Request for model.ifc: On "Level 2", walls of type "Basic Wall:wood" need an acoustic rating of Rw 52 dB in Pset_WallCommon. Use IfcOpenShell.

First a look at what the model holds.

```python
import ifcopenshell
import ifcopenshell.util.element

model = ifcopenshell.open("model.ifc")
print(model.schema)
storey = next(s for s in model.by_type("IfcBuildingStorey") if s.Name == "Level 2")
walls = [e for e in ifcopenshell.util.element.get_decomposition(storey) if e.is_a("IfcWall")]
seen = {}
for e in walls:
    element_type = ifcopenshell.util.element.get_type(e)
    key = (element_type.Name if element_type != e and element_type else None, ifcopenshell.util.element.get_pset(e, "Pset_WallCommon", "AcousticRating"))
    seen[key] = seen.get(key, 0) + 1
for (name, value), count in sorted(seen.items(), key=str):
    print(count, "x", name, "|", value)
```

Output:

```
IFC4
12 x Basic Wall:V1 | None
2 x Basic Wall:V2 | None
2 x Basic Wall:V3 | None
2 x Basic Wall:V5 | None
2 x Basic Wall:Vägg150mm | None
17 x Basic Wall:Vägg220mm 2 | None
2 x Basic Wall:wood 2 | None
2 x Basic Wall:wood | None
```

```python
import ifcopenshell
import ifcopenshell.api.pset
import ifcopenshell.util.element

model = ifcopenshell.open("model.ifc")

storey = next(s for s in model.by_type("IfcBuildingStorey") if s.Name == "Level 2")
walls = [e for e in ifcopenshell.util.element.get_decomposition(storey) if e.is_a("IfcWall")]

count = 0
for e in walls:
    element_type = ifcopenshell.util.element.get_type(e)
    if element_type in (None, e) or element_type.Name != "Basic Wall:wood":
        continue
    # add_pset returns the element's existing set when there is one.
    pset = ifcopenshell.api.pset.add_pset(model, product=e, name="Pset_WallCommon")
    ifcopenshell.api.pset.edit_pset(model, pset=pset, properties={"AcousticRating": "Rw 52 dB"})
    count += 1

print(count, "walls updated")

model.write("model_edited.ifc")
```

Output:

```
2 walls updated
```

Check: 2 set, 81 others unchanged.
